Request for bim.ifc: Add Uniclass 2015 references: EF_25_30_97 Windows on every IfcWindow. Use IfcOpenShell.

First a look at what the model holds.

```python
import ifcopenshell

model = ifcopenshell.open("bim.ifc")
print(model.schema)
print("classifications:", [c.Name for c in model.by_type("IfcClassification")])
for ifc_class in ("IfcDoor", "IfcRoof", "IfcStair", "IfcWall", "IfcWindow"):
    print(ifc_class, len(model.by_type(ifc_class)))
```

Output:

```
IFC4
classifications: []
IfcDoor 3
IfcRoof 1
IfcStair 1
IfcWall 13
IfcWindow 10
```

```python
import ifcopenshell
import ifcopenshell.api.classification

model = ifcopenshell.open("bim.ifc")

system = ifcopenshell.api.classification.add_classification(model, classification="Uniclass 2015")

codes = {
    "IfcWindow": ("EF_25_30_97", "Windows"),
}
for ifc_class, (code, name) in codes.items():
    products = model.by_type(ifc_class)
    ifcopenshell.api.classification.add_reference(
        model, products=products, classification=system, identification=code, name=name
    )
    print(code, len(products))

model.write("bim-out.ifc")
```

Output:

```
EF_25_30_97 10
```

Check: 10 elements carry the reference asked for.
